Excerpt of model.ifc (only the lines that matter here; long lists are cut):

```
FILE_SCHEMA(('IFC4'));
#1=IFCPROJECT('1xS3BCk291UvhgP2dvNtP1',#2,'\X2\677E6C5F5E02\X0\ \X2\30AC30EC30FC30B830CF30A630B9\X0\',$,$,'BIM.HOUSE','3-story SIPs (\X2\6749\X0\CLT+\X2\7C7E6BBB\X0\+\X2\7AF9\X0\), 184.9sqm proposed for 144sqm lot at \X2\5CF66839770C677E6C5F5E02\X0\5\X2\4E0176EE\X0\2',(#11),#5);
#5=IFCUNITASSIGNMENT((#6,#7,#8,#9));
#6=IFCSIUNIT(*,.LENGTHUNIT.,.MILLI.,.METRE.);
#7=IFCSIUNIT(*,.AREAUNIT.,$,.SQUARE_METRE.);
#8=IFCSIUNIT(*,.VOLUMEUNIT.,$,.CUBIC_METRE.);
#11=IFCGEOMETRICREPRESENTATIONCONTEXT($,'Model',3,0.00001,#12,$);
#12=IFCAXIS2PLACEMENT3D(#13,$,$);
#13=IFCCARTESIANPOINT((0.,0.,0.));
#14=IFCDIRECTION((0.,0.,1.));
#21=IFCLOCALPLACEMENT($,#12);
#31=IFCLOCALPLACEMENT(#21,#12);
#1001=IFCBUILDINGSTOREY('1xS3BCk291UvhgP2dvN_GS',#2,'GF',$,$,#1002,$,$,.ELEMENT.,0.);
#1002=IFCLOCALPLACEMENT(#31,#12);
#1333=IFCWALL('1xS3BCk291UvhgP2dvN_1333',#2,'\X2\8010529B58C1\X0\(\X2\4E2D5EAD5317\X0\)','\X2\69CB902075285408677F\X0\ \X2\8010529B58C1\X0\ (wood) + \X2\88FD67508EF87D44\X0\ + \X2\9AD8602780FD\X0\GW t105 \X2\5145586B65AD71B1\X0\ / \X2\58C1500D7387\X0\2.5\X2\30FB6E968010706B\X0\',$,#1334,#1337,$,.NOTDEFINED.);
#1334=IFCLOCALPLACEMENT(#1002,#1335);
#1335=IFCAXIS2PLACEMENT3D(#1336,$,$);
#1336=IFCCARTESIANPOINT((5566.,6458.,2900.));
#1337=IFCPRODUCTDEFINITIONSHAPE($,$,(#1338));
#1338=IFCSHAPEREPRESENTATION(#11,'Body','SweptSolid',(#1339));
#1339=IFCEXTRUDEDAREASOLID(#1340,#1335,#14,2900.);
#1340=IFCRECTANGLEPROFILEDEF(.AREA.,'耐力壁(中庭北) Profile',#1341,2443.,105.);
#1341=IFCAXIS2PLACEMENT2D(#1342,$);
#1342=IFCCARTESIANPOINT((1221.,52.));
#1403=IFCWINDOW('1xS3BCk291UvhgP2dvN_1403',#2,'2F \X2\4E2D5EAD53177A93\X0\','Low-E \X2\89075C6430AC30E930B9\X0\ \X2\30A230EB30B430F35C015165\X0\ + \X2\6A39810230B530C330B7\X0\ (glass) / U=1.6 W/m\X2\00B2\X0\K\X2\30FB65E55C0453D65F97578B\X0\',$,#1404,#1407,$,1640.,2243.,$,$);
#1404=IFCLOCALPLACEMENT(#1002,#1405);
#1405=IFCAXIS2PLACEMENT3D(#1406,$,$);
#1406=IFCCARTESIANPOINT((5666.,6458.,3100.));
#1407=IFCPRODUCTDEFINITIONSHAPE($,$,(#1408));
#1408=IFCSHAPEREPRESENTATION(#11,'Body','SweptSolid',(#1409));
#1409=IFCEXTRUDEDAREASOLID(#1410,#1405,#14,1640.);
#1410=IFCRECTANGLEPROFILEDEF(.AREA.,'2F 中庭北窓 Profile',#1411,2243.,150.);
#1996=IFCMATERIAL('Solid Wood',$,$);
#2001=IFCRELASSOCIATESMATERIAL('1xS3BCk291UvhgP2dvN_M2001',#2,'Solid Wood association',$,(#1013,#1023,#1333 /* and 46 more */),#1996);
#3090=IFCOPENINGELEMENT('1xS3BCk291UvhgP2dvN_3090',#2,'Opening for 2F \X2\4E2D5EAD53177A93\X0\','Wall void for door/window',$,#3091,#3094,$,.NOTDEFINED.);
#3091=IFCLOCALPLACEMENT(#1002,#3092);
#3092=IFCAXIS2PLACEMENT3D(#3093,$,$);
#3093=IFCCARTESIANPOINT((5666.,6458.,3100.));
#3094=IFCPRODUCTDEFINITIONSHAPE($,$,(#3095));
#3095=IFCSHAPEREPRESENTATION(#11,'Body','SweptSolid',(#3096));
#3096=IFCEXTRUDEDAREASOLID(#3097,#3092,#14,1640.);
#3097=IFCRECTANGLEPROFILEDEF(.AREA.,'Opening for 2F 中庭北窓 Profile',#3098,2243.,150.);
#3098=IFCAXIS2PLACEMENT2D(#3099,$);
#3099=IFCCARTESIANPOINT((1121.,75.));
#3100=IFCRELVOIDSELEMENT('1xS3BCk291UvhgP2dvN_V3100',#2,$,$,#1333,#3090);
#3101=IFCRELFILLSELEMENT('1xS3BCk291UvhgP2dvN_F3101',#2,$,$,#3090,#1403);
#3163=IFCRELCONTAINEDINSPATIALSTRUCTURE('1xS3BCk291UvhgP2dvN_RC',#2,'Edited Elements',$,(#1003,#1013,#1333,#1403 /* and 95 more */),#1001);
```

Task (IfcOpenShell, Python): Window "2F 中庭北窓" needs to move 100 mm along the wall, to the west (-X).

```python
import ifcopenshell
import ifcopenshell.api.geometry
import ifcopenshell.util.placement
import ifcopenshell.util.unit

model = ifcopenshell.open("model.ifc")
unit_scale = ifcopenshell.util.unit.calculate_unit_scale(model)

window = model.by_guid("1xS3BCk291UvhgP2dvN_1403")
opening = window.FillsVoids[0].RelatingOpeningElement
wall = opening.VoidsElements[0].RelatingBuildingElement

wall_matrix = ifcopenshell.util.placement.get_local_placement(wall.ObjectPlacement)
shift = wall_matrix[:3, 0] * -0.1 / unit_scale
before = ifcopenshell.util.placement.get_local_placement(window.ObjectPlacement)[:3, 3].copy()

# The window is not placed relative to its opening, so move both.
for product in (opening, window):
    matrix = ifcopenshell.util.placement.get_local_placement(product.ObjectPlacement)
    matrix[:3, 3] += shift
    ifcopenshell.api.geometry.edit_object_placement(model, product=product, matrix=matrix, is_si=False)

after = ifcopenshell.util.placement.get_local_placement(window.ObjectPlacement)[:3, 3]
print("window moved by", (after - before).round(3) + 0.0)

model.write("model_v2.ifc")
```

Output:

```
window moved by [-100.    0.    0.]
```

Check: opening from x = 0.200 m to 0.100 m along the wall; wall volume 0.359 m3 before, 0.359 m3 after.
